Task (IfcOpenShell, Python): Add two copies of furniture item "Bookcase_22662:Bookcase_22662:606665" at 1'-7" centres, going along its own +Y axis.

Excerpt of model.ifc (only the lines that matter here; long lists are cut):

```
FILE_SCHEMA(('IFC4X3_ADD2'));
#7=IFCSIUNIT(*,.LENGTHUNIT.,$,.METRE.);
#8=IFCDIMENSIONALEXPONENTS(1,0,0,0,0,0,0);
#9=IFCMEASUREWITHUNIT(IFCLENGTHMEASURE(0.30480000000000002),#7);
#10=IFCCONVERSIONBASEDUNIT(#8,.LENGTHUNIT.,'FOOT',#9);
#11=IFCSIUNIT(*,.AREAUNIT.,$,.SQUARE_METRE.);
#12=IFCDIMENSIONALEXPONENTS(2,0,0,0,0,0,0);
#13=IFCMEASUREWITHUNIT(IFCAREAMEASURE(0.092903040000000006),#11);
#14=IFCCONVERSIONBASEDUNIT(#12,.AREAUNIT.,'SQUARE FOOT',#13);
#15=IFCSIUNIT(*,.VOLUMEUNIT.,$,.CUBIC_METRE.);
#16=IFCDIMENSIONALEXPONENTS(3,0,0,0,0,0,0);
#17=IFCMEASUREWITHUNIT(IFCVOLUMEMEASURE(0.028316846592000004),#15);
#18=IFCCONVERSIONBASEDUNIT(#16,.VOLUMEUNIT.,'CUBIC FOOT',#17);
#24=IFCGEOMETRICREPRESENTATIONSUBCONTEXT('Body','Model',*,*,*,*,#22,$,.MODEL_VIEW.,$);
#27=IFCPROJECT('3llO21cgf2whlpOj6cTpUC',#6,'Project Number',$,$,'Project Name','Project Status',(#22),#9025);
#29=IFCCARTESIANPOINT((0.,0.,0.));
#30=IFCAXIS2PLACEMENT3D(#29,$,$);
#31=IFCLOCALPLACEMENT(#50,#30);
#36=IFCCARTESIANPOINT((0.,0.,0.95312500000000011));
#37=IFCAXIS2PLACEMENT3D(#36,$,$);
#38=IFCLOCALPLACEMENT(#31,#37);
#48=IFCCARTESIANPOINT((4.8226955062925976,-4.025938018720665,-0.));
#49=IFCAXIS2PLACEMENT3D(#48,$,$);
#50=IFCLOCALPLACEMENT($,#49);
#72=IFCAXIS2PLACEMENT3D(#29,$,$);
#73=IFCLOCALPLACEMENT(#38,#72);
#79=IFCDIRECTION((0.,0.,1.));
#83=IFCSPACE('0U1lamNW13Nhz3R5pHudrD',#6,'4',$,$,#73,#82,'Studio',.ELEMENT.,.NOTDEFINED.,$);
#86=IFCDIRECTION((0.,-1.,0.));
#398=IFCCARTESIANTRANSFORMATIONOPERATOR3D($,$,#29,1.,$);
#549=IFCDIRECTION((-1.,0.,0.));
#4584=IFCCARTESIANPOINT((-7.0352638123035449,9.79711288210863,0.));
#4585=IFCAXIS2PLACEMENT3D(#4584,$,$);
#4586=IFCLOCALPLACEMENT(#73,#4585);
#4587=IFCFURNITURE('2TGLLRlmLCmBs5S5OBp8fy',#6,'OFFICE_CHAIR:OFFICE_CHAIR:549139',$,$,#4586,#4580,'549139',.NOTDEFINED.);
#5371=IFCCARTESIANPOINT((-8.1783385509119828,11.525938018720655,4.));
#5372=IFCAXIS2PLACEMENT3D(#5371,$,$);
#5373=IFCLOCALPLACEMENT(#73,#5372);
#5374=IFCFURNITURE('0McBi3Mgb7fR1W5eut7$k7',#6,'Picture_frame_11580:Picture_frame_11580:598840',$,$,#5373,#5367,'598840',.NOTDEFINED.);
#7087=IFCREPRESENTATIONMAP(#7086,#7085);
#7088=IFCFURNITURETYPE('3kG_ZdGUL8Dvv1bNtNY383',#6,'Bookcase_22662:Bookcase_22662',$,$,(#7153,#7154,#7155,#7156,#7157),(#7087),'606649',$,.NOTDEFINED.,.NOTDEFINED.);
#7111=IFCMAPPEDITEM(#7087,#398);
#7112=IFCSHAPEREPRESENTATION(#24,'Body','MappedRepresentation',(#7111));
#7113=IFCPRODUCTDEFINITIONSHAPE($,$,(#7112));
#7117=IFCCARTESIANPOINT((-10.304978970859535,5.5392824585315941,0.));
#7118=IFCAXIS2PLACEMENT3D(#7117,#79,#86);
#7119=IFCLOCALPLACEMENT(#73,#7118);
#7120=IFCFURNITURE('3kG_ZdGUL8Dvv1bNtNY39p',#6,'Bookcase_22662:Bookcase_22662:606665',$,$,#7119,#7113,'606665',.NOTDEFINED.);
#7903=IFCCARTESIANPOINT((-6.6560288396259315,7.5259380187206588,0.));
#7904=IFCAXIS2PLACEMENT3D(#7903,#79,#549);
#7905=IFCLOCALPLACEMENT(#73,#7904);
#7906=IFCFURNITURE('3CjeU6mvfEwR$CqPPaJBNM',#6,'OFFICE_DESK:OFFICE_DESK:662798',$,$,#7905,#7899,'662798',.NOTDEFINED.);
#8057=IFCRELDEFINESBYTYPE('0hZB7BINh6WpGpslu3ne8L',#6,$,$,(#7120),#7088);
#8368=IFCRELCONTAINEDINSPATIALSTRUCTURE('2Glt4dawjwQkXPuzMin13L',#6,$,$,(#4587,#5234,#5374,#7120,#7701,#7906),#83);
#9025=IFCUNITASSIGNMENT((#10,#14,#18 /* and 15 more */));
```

```python
import ifcopenshell
import ifcopenshell.api.geometry
import ifcopenshell.api.root
import ifcopenshell.util.element
import ifcopenshell.util.placement
import ifcopenshell.util.unit

model = ifcopenshell.open("model.ifc")
unit_scale = ifcopenshell.util.unit.calculate_unit_scale(model)


def reuse_history(source, copy):
    """copy_class also copies each property set's owner history, people and application; keep the originals."""
    for rel in copy.IsDefinedBy:
        if rel.is_a("IfcRelDefinesByProperties") and (history := rel.RelatingPropertyDefinition.OwnerHistory):
            rel.RelatingPropertyDefinition.OwnerHistory = source.OwnerHistory
            ifcopenshell.util.element.remove_deep2(model, history)


source = model.by_guid("3kG_ZdGUL8Dvv1bNtNY39p")
base = ifcopenshell.util.placement.get_local_placement(source.ObjectPlacement)
step = base[:3, 1] * 19 * 0.0254 / unit_scale

for i in range(1, 3):
    copy = ifcopenshell.api.root.copy_class(model, product=source)
    copy.Representation = ifcopenshell.util.element.copy_deep(
        model, source.Representation, exclude=["IfcGeometricRepresentationContext", "IfcRepresentationMap"]
    )
    copy.Name = "Bookcase_22662:Bookcase_22662"
    copy.Tag = None
    reuse_history(source, copy)
    matrix = base.copy()
    matrix[:3, 3] += i * step
    print("added at", matrix[:3, 3].round(3) + 0.0)
    ifcopenshell.api.geometry.edit_object_placement(model, product=copy, matrix=matrix, is_si=False)

model.write("model_rev.ifc")
```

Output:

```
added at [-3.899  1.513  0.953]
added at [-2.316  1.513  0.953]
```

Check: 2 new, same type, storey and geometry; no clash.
